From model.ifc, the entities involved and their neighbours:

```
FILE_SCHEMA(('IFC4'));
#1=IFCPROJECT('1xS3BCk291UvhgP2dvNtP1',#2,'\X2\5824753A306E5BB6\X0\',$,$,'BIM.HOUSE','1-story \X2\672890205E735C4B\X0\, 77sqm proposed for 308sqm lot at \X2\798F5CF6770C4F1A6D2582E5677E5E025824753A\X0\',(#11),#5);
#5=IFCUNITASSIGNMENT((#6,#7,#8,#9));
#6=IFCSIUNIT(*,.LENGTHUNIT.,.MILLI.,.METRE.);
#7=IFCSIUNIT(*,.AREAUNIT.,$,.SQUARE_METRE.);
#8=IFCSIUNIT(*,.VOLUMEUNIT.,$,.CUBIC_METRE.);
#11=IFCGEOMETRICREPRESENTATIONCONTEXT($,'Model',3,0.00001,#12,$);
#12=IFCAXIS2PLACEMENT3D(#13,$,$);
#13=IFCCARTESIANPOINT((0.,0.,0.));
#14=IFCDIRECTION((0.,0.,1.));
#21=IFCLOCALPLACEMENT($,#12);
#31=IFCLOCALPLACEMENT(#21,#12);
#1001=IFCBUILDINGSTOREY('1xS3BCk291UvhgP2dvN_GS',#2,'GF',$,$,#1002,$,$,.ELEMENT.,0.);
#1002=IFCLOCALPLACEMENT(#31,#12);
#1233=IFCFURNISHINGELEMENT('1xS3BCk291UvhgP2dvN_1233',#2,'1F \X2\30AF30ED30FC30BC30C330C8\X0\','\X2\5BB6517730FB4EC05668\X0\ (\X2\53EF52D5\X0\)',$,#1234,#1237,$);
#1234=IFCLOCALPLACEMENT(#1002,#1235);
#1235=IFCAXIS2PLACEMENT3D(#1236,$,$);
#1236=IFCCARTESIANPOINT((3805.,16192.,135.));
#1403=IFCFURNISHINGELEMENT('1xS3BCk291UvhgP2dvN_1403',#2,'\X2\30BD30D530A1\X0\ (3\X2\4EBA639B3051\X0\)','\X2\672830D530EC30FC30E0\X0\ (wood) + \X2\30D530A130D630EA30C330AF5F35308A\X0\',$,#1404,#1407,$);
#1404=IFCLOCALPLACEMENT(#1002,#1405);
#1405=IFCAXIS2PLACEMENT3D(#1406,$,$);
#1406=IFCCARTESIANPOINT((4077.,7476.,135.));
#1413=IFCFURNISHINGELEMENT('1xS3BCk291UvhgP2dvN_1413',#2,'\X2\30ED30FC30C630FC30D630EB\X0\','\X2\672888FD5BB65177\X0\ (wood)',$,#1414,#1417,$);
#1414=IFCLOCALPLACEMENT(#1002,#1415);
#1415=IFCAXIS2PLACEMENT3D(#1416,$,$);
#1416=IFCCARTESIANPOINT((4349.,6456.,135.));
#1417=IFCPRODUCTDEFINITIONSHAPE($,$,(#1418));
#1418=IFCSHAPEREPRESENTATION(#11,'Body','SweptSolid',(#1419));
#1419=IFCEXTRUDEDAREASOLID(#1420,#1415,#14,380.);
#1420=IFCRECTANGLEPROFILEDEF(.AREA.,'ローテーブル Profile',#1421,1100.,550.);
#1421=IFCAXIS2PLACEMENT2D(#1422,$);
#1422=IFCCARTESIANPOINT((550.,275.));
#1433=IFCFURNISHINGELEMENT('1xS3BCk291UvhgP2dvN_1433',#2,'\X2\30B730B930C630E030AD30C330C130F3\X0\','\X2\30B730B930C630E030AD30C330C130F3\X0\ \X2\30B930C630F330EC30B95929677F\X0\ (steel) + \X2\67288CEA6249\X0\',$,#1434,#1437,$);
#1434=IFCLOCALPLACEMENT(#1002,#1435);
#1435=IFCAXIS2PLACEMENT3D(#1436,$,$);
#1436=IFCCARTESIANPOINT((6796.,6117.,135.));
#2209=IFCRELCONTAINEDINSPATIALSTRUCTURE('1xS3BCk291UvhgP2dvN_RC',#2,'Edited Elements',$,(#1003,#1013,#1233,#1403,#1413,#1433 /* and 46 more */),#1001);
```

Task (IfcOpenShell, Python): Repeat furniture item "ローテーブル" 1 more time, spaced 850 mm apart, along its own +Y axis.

```python
import ifcopenshell
import ifcopenshell.api.geometry
import ifcopenshell.api.root
import ifcopenshell.util.element
import ifcopenshell.util.placement
import ifcopenshell.util.unit

model = ifcopenshell.open("model.ifc")
unit_scale = ifcopenshell.util.unit.calculate_unit_scale(model)


def reuse_history(source, copy):
    """copy_class also copies each property set's owner history, people and application; keep the originals."""
    for rel in copy.IsDefinedBy:
        if rel.is_a("IfcRelDefinesByProperties") and (history := rel.RelatingPropertyDefinition.OwnerHistory):
            rel.RelatingPropertyDefinition.OwnerHistory = source.OwnerHistory
            ifcopenshell.util.element.remove_deep2(model, history)


source = model.by_guid("1xS3BCk291UvhgP2dvN_1413")
base = ifcopenshell.util.placement.get_local_placement(source.ObjectPlacement)
step = base[:3, 1] * 0.85 / unit_scale

for i in range(1, 2):
    copy = ifcopenshell.api.root.copy_class(model, product=source)
    copy.Representation = ifcopenshell.util.element.copy_deep(
        model, source.Representation, exclude=["IfcGeometricRepresentationContext", "IfcRepresentationMap"]
    )
    reuse_history(source, copy)
    matrix = base.copy()
    matrix[:3, 3] += i * step
    print("added at", matrix[:3, 3].round(3) + 0.0)
    ifcopenshell.api.geometry.edit_object_placement(model, product=copy, matrix=matrix, is_si=False)

model.write("model-out.ifc")
```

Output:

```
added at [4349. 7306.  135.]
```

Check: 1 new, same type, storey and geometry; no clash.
